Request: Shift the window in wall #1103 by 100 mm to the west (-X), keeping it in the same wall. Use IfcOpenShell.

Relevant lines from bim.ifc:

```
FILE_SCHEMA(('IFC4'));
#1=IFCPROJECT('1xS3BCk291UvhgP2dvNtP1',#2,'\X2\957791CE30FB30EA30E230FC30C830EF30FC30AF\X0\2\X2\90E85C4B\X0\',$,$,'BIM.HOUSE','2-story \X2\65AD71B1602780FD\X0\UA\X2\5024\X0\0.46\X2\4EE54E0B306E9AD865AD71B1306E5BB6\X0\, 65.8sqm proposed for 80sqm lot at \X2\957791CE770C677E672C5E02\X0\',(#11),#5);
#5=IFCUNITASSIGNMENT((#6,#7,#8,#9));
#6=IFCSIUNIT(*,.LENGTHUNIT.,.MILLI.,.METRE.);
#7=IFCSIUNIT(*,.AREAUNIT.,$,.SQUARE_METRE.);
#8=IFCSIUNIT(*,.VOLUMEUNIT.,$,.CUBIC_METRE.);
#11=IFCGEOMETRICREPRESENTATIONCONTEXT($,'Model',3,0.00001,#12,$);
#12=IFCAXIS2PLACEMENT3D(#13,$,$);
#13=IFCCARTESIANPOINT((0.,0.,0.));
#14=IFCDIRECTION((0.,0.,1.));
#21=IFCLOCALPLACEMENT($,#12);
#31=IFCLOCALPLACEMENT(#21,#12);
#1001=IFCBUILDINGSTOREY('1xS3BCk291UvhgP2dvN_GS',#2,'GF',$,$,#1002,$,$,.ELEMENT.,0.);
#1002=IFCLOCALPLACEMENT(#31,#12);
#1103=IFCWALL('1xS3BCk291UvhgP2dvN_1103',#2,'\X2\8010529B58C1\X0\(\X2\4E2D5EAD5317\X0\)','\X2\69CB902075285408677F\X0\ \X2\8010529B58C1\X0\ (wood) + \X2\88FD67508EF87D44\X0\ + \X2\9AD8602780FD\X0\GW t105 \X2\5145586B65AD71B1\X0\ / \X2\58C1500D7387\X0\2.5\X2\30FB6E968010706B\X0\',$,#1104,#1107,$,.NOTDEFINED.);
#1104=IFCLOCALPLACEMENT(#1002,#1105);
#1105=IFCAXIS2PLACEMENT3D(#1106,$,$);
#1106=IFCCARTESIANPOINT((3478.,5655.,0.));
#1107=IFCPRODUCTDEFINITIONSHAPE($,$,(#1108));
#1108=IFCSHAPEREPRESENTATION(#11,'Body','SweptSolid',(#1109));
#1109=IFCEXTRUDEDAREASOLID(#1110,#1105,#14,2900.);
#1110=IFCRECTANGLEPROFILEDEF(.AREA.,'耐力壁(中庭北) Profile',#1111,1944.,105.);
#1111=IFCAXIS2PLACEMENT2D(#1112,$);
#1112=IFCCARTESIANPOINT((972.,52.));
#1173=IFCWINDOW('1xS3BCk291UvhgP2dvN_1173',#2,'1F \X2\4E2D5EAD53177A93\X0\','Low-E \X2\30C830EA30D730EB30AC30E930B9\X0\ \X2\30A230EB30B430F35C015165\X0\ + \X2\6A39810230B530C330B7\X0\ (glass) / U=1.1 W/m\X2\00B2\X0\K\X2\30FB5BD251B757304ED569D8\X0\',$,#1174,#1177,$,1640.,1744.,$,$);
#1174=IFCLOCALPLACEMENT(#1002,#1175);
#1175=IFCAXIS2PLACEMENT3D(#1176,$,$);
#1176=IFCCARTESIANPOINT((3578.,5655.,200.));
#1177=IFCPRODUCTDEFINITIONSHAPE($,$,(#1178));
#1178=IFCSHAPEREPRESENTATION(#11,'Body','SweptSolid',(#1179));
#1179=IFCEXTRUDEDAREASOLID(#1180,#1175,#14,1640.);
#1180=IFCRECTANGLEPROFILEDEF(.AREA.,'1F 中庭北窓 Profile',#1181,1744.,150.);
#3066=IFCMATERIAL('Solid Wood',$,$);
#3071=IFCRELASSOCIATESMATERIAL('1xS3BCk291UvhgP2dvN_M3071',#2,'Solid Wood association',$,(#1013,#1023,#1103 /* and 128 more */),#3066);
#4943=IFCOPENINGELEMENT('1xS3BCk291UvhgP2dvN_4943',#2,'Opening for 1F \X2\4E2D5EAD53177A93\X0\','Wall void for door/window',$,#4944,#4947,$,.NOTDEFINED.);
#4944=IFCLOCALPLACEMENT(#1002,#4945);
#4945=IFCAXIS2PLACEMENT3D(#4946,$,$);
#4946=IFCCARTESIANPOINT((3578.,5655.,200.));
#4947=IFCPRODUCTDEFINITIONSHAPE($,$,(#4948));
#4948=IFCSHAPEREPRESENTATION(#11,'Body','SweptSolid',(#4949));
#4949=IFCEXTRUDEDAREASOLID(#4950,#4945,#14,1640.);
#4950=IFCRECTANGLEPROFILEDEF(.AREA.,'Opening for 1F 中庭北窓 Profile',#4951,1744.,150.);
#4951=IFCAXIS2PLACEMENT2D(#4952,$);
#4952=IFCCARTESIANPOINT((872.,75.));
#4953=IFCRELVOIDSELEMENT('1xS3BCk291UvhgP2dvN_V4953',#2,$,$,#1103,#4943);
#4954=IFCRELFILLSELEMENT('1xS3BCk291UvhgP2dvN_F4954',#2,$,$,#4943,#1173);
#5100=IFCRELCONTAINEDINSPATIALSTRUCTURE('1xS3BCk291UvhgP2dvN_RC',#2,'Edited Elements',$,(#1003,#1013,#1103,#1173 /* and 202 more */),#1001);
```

```python
import ifcopenshell
import ifcopenshell.api.geometry
import ifcopenshell.util.placement

model = ifcopenshell.open("bim.ifc")

window = model.by_id(1173)
opening = window.FillsVoids[0].RelatingOpeningElement
wall = opening.VoidsElements[0].RelatingBuildingElement

wall_matrix = ifcopenshell.util.placement.get_local_placement(wall.ObjectPlacement)
shift = wall_matrix[:3, 0] * -100.0
before = ifcopenshell.util.placement.get_local_placement(window.ObjectPlacement)[:3, 3].copy()

# The window is not placed relative to its opening, so move both.
for product in (opening, window):
    matrix = ifcopenshell.util.placement.get_local_placement(product.ObjectPlacement)
    matrix[:3, 3] += shift
    ifcopenshell.api.geometry.edit_object_placement(model, product=product, matrix=matrix, is_si=False)

after = ifcopenshell.util.placement.get_local_placement(window.ObjectPlacement)[:3, 3]
print("window moved by", (after - before).round(3) + 0.0)

model.write("bim_v2.ifc")
```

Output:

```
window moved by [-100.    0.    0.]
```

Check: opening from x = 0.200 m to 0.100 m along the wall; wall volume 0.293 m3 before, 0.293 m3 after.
